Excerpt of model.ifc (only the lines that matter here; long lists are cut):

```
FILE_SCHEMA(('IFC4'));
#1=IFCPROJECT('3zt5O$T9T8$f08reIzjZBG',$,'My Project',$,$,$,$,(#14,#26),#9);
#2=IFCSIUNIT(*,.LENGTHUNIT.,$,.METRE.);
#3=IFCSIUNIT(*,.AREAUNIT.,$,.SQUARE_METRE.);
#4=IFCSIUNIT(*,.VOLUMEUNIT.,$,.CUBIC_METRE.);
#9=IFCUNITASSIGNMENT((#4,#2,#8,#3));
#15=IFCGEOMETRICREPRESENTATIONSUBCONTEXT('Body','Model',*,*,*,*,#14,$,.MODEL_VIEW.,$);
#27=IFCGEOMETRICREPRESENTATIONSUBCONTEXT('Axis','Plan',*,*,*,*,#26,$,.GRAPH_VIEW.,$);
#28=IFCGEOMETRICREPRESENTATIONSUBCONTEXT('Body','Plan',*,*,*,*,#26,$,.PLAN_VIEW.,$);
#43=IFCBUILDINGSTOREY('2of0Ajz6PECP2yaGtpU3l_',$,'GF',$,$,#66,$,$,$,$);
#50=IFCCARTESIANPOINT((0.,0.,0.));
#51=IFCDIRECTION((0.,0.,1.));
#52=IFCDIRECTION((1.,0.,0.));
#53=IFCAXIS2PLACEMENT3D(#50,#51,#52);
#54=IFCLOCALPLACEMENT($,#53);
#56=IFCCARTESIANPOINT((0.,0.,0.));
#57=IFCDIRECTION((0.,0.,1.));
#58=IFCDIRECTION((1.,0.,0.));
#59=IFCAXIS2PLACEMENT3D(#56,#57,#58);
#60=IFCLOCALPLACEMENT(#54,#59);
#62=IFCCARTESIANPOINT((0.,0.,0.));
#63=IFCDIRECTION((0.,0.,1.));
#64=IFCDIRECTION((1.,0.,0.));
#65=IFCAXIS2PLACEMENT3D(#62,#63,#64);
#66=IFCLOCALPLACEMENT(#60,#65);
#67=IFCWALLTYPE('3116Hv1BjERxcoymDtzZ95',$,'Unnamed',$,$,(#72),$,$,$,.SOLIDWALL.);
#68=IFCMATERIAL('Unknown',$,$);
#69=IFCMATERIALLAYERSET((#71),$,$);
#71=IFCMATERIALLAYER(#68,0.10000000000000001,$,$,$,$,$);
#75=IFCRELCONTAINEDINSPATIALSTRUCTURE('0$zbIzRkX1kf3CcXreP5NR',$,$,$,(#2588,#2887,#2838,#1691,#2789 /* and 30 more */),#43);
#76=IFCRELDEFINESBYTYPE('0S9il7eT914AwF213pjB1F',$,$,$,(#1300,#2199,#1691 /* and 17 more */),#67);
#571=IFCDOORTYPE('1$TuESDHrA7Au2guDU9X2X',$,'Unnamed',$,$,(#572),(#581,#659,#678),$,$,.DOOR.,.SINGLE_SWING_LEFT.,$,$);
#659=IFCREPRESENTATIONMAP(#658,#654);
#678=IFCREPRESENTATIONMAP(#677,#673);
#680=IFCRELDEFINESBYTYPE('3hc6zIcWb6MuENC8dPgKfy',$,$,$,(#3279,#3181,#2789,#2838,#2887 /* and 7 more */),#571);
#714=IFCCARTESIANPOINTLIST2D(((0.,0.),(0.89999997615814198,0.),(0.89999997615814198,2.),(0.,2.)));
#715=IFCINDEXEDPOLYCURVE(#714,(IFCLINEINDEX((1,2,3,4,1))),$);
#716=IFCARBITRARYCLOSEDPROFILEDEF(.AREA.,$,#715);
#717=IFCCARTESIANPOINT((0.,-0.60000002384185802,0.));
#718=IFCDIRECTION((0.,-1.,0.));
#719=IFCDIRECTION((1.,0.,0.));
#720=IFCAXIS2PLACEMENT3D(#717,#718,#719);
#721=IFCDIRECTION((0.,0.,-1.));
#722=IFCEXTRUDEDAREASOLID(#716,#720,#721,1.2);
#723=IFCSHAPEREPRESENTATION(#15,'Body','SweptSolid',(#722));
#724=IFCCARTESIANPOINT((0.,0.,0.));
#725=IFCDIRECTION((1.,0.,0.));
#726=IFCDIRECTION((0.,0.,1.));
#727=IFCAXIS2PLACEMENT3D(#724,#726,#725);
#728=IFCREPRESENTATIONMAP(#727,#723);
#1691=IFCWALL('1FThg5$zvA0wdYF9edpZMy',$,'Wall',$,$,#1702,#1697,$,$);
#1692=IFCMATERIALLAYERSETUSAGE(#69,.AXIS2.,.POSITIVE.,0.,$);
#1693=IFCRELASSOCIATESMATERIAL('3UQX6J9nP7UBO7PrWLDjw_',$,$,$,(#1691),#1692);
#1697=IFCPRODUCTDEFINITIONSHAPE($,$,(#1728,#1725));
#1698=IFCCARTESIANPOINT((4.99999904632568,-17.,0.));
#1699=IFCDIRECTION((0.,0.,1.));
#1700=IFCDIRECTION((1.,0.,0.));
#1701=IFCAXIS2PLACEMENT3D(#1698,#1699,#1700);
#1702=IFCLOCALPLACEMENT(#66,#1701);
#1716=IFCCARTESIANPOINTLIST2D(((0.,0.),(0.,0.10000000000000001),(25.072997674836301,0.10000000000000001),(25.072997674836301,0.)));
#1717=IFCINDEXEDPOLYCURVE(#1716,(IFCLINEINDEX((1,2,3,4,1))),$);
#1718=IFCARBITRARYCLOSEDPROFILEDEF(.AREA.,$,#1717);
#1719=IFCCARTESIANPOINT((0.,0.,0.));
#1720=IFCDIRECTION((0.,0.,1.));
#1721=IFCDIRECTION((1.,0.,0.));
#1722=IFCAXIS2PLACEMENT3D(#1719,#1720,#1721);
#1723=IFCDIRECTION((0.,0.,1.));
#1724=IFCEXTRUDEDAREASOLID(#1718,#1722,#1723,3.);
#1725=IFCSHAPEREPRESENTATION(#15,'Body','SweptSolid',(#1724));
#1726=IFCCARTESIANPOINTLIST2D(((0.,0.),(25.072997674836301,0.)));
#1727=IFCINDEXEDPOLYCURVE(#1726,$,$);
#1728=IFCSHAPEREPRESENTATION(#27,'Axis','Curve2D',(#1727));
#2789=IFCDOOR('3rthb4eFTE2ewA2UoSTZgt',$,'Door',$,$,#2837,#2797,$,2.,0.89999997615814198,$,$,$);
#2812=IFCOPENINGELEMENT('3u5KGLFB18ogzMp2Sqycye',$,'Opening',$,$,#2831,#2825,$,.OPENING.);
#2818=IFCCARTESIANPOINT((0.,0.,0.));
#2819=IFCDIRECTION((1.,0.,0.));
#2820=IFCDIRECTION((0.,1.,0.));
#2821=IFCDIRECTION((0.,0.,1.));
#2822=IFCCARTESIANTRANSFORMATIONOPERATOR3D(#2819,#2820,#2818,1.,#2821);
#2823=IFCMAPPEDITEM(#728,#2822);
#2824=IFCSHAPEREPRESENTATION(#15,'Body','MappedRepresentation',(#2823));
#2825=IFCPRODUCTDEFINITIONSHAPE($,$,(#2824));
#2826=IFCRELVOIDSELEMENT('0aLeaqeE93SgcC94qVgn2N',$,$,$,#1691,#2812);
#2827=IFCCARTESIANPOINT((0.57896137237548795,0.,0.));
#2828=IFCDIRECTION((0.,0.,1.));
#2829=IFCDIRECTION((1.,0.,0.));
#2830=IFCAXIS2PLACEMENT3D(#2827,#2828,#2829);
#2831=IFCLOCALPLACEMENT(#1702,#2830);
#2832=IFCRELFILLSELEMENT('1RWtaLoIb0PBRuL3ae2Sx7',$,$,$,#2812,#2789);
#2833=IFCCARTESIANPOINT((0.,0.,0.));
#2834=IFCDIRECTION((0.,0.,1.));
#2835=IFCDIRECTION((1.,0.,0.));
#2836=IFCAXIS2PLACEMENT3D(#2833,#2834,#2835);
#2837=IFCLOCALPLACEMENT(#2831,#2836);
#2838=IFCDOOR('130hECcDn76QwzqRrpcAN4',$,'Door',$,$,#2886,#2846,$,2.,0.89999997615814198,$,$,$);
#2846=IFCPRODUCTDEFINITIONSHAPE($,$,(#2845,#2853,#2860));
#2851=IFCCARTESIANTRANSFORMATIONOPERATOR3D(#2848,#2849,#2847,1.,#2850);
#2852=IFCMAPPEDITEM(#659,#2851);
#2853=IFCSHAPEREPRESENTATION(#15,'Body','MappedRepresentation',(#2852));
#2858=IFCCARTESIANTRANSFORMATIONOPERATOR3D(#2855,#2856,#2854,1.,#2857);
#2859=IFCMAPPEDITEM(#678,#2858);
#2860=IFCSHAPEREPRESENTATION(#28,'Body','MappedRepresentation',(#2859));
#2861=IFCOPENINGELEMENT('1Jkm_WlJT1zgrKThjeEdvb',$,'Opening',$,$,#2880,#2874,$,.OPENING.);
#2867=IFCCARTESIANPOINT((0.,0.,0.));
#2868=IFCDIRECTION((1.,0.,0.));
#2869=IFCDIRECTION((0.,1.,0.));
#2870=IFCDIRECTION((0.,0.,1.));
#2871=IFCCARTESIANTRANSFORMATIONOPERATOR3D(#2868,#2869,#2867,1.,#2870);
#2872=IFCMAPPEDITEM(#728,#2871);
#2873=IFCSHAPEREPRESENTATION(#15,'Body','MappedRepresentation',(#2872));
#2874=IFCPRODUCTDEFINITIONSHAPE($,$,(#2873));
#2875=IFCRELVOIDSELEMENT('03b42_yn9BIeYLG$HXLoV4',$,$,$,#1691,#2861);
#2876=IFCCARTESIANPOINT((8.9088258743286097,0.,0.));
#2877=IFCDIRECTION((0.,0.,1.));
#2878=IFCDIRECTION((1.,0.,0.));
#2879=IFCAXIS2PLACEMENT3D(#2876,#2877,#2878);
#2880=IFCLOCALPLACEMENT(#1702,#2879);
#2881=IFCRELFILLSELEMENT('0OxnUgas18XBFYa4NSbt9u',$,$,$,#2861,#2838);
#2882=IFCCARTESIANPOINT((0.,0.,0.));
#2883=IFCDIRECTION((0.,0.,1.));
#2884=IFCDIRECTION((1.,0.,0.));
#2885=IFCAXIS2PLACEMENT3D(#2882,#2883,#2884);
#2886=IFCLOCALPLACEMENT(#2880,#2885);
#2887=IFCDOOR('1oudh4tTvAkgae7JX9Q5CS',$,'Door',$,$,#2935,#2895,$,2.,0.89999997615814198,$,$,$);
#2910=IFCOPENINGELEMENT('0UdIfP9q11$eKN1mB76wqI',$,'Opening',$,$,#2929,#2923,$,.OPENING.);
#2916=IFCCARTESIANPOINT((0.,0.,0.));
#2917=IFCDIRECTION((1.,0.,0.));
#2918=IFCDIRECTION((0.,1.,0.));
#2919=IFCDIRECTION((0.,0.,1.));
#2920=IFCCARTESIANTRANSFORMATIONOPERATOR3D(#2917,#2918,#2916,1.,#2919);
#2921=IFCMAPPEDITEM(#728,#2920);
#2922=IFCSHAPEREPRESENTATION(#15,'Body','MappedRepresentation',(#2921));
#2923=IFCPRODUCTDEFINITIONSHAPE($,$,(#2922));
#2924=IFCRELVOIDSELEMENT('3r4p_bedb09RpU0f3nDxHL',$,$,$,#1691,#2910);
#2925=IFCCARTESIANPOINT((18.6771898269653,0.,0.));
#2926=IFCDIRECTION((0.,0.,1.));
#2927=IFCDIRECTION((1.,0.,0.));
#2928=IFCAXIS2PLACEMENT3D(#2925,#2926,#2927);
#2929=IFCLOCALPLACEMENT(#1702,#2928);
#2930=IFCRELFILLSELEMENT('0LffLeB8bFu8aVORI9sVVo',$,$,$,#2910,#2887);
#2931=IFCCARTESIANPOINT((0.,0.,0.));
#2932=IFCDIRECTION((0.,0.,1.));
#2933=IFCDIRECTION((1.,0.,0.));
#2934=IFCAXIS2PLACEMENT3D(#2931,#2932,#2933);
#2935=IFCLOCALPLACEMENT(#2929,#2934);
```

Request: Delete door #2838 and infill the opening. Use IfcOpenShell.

```python
import ifcopenshell
import ifcopenshell.api.feature
import ifcopenshell.api.root
import ifcopenshell.geom
import ifcopenshell.util.shape

model = ifcopenshell.open("model.ifc")
settings = ifcopenshell.geom.settings()


def volume(element):
    """Net volume in cubic metres, openings subtracted."""
    shape = ifcopenshell.geom.create_shape(settings, element)
    return ifcopenshell.util.shape.get_volume(shape.geometry)


door = model.by_guid("130hECcDn76QwzqRrpcAN4")
opening = door.FillsVoids[0].RelatingOpeningElement
wall = opening.VoidsElements[0].RelatingBuildingElement
before = volume(wall)

ifcopenshell.api.root.remove_product(model, product=door)
ifcopenshell.api.feature.remove_feature(model, feature=opening)

after = volume(wall)

print(f"wall volume {before:.3f} -> {after:.3f} m3")

model.write("model_v2.ifc")
```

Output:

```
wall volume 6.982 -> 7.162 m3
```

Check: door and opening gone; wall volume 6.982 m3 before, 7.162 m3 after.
